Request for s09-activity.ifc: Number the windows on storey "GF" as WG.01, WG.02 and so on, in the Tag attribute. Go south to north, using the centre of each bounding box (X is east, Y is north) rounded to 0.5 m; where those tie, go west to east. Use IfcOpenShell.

First a look at what the model holds.

```python
import ifcopenshell
import ifcopenshell.util.element
import ifcopenshell.util.placement

model = ifcopenshell.open("s09-activity.ifc")
print(model.schema)
storey = next(s for s in model.by_type("IfcBuildingStorey") if s.Name == "GF")
windows = [e for e in ifcopenshell.util.element.get_decomposition(storey) if e.is_a("IfcWindow")]
for e in sorted(windows, key=lambda e: e.id()):
    origin = ifcopenshell.util.placement.get_local_placement(e.ObjectPlacement)[:3, 3]
    print(e.id(), e.Tag, e.Name, origin.round(2) + 0.0, sep=" | ")
```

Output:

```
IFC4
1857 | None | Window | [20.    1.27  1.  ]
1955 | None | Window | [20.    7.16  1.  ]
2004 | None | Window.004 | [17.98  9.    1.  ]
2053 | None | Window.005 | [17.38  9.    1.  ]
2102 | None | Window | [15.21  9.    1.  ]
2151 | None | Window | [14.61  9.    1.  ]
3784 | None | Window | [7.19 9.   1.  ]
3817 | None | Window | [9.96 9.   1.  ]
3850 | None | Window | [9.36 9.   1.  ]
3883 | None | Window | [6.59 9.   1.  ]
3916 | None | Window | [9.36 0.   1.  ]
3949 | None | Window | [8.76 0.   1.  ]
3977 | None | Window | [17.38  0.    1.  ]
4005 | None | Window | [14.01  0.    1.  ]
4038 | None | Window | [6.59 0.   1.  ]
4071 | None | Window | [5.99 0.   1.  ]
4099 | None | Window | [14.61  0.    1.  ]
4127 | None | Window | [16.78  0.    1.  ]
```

```python
import ifcopenshell
import ifcopenshell.geom
import ifcopenshell.util.element
import ifcopenshell.util.shape

model = ifcopenshell.open("s09-activity.ifc")
settings = ifcopenshell.geom.settings()
settings.set("use-world-coords", True)


def centre(element):
    shape = ifcopenshell.geom.create_shape(settings, element)
    return ifcopenshell.util.shape.get_bbox_centroid(shape.geometry)


storey = next(s for s in model.by_type("IfcBuildingStorey") if s.Name == "GF")
windows = [e for e in ifcopenshell.util.element.get_decomposition(storey) if e.is_a("IfcWindow")]

# Insertion points can sit at a corner or the storey origin, so sort by the geometry (in metres).
centres = {e: centre(e) for e in windows}
windows.sort(key=lambda e: (round(centres[e][1] / 0.5), centres[e][0]))

for i, e in enumerate(windows, start=1):
    number = f"WG.{i:02d}"
    e.Tag = number
    print(e.id(), number)

model.write("s09-activity_rev.ifc")
```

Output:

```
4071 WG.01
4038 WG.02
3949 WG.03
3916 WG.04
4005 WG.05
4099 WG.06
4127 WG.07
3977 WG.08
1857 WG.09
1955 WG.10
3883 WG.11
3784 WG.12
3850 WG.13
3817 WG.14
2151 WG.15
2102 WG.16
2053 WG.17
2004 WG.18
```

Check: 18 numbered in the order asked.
